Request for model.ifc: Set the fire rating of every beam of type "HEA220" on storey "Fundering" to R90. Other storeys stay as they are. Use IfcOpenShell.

First a look at what the model holds.

```python
import ifcopenshell
import ifcopenshell.util.element

model = ifcopenshell.open("model.ifc")
print(model.schema)
storey = next(s for s in model.by_type("IfcBuildingStorey") if s.Name == "Fundering")
beams = [e for e in ifcopenshell.util.element.get_decomposition(storey) if e.is_a("IfcBeam")]
seen = {}
for e in beams:
    element_type = ifcopenshell.util.element.get_type(e)
    key = (element_type.Name if element_type != e and element_type else None, ifcopenshell.util.element.get_pset(e, "Pset_BeamCommon", "FireRating"))
    seen[key] = seen.get(key, 0) + 1
for (name, value), count in sorted(seen.items(), key=str):
    print(count, "x", name, "|", value)
```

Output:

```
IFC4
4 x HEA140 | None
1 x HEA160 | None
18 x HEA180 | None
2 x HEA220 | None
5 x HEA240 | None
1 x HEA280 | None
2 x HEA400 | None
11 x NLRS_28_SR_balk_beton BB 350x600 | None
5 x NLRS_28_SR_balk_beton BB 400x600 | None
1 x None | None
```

```python
import ifcopenshell
import ifcopenshell.api.pset
import ifcopenshell.util.element

model = ifcopenshell.open("model.ifc")

storey = next(s for s in model.by_type("IfcBuildingStorey") if s.Name == "Fundering")
beams = [e for e in ifcopenshell.util.element.get_decomposition(storey) if e.is_a("IfcBeam")]

count = 0
for e in beams:
    element_type = ifcopenshell.util.element.get_type(e)
    if element_type in (None, e) or element_type.Name != "HEA220":
        continue
    # add_pset returns the element's existing set when there is one.
    pset = ifcopenshell.api.pset.add_pset(model, product=e, name="Pset_BeamCommon")
    ifcopenshell.api.pset.edit_pset(model, pset=pset, properties={"FireRating": "R90"})
    count += 1

print(count, "beams updated")

model.write("model_edited.ifc")
```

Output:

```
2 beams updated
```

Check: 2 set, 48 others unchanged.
